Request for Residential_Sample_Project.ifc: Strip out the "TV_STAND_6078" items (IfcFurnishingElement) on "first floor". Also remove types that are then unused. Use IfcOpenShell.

First a look at what the model holds.

```python
import ifcopenshell
import ifcopenshell.util.element

model = ifcopenshell.open("Residential_Sample_Project.ifc")
print(model.schema)
storey = next(s for s in model.by_type("IfcBuildingStorey") if s.Name == "first floor")
furniture = [e for e in ifcopenshell.util.element.get_decomposition(storey) if e.is_a("IfcFurnishingElement")]
seen = {}
for e in furniture:
    element_type = ifcopenshell.util.element.get_type(e)
    name = element_type.Name if element_type not in (None, e) else None
    seen[name] = seen.get(name, 0) + 1
for name, count in sorted(seen.items(), key=str):
    print(count, "x", name)
```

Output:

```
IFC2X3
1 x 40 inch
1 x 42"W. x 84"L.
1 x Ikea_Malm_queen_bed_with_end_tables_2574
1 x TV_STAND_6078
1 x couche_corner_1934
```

```python
import ifcopenshell
import ifcopenshell.api.root
import ifcopenshell.util.element

model = ifcopenshell.open("Residential_Sample_Project.ifc")

storey = next(s for s in model.by_type("IfcBuildingStorey") if s.Name == "first floor")
furniture = [e for e in ifcopenshell.util.element.get_decomposition(storey) if e.is_a("IfcFurnishingElement")]
targets = [e for e in furniture if (t := ifcopenshell.util.element.get_type(e)) not in (None, e) and t.Name == "TV_STAND_6078"]
types = {ifcopenshell.util.element.get_type(e) for e in targets} - {None, *targets}

for e in targets:
    ifcopenshell.api.root.remove_product(model, product=e)
print(len(targets), "removed")

unused = [t for t in types if not ifcopenshell.util.element.get_types(t)]
for t in unused:
    ifcopenshell.api.root.remove_product(model, product=t)
print(len(unused), "unused types removed")

model.write("Residential_Sample_Project_v2.ifc")
```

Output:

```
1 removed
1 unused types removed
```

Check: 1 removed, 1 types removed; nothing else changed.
